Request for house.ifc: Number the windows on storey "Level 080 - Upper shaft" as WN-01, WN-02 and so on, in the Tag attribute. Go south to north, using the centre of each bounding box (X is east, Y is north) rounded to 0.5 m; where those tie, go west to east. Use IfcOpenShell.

First a look at what the model holds.

```python
import ifcopenshell
import ifcopenshell.util.element
import ifcopenshell.util.placement

model = ifcopenshell.open("house.ifc")
print(model.schema)
storey = next(s for s in model.by_type("IfcBuildingStorey") if s.Name == "Level 080 - Upper shaft")
windows = [e for e in ifcopenshell.util.element.get_decomposition(storey) if e.is_a("IfcWindow")]
for e in sorted(windows, key=lambda e: e.id()):
    origin = ifcopenshell.util.placement.get_local_placement(e.ObjectPlacement)[:3, 3]
    print(e.id(), e.Tag, e.Name, origin.round(2) + 0.0, sep=" | ")
```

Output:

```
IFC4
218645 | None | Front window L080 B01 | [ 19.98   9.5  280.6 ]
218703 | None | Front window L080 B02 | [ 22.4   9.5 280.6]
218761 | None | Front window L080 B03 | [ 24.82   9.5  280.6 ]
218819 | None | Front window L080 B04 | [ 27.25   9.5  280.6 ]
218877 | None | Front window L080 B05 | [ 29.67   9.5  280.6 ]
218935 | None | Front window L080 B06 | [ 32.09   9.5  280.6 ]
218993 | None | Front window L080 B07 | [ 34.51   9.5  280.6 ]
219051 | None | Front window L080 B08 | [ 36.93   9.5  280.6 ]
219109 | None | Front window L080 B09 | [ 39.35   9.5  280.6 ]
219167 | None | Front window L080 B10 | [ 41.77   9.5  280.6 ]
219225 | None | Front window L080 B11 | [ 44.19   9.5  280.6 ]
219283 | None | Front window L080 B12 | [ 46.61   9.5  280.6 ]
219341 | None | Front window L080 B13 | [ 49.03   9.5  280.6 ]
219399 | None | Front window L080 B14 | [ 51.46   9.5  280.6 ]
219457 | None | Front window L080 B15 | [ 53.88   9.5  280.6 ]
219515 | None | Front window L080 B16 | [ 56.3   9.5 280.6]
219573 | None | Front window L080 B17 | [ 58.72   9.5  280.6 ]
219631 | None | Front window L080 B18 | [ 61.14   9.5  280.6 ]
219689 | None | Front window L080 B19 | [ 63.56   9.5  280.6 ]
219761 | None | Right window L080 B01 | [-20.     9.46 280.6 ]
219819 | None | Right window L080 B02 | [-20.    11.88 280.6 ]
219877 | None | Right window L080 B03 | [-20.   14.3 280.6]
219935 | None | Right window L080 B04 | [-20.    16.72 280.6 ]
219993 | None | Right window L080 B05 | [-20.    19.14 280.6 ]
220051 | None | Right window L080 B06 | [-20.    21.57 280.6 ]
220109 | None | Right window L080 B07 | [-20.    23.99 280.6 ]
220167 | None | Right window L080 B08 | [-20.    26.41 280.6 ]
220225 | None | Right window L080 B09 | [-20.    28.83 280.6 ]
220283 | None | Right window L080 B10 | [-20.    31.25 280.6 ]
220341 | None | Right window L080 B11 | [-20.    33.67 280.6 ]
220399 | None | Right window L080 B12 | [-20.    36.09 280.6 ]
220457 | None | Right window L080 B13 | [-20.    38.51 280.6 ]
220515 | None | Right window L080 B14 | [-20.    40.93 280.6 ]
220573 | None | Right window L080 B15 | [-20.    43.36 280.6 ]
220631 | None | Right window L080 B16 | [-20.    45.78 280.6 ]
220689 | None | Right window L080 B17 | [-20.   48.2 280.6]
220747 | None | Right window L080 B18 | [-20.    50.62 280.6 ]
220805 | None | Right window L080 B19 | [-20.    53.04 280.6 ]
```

```python
import ifcopenshell
import ifcopenshell.geom
import ifcopenshell.util.element
import ifcopenshell.util.shape

model = ifcopenshell.open("house.ifc")
settings = ifcopenshell.geom.settings()
settings.set("use-world-coords", True)


def centre(element):
    shape = ifcopenshell.geom.create_shape(settings, element)
    return ifcopenshell.util.shape.get_bbox_centroid(shape.geometry)


storey = next(s for s in model.by_type("IfcBuildingStorey") if s.Name == "Level 080 - Upper shaft")
windows = [e for e in ifcopenshell.util.element.get_decomposition(storey) if e.is_a("IfcWindow")]

# Insertion points can sit at a corner or the storey origin, so sort by the geometry (in metres).
centres = {e: centre(e) for e in windows}
windows.sort(key=lambda e: (round(centres[e][1] / 0.5), centres[e][0]))

for i, e in enumerate(windows, start=1):
    number = f"WN-{i:02d}"
    e.Tag = number
    print(e.id(), number)

model.write("house-out.ifc")
```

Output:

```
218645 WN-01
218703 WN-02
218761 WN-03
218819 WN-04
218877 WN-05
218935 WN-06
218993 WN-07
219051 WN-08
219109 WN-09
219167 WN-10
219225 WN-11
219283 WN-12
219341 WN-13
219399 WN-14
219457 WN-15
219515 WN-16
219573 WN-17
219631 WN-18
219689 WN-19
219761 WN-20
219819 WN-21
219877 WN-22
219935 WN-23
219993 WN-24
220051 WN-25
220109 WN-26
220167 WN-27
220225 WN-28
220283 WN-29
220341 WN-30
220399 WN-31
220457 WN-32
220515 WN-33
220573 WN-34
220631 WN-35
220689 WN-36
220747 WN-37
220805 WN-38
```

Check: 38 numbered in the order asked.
